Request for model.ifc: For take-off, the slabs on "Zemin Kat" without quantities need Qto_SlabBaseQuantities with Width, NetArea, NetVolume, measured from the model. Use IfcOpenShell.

First a look at what the model holds.

```python
import ifcopenshell
import ifcopenshell.util.element
import ifcopenshell.util.unit

model = ifcopenshell.open("model.ifc")
print(model.schema)
for unit_type in ("LENGTHUNIT", "AREAUNIT", "VOLUMEUNIT"):
    print(unit_type, ifcopenshell.util.unit.calculate_unit_scale(model, unit_type))
storey = next(s for s in model.by_type("IfcBuildingStorey") if s.Name == "Zemin Kat")
slabs = [e for e in ifcopenshell.util.element.get_decomposition(storey) if e.is_a("IfcSlab")]
for e in sorted(slabs, key=lambda e: e.id()):
    print(e.id(), e.is_a(), e.Name, list(ifcopenshell.util.element.get_psets(e, qtos_only=True)), sep=" | ")
```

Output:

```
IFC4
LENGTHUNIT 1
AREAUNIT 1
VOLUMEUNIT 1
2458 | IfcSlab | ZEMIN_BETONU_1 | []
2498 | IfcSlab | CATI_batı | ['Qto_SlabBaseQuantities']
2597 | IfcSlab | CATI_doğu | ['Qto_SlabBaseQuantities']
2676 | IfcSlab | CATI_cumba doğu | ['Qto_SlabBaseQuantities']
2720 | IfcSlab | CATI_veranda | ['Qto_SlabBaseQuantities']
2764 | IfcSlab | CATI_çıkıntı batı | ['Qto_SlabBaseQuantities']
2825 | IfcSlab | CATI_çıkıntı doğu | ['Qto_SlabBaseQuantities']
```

```python
import ifcopenshell
import ifcopenshell.api.pset
import ifcopenshell.geom
import ifcopenshell.util.element
import ifcopenshell.util.shape
import ifcopenshell.util.unit

model = ifcopenshell.open("model.ifc")
unit_scale = ifcopenshell.util.unit.calculate_unit_scale(model)
area_scale = ifcopenshell.util.unit.calculate_unit_scale(model, "AREAUNIT")
volume_scale = ifcopenshell.util.unit.calculate_unit_scale(model, "VOLUMEUNIT")
settings = ifcopenshell.geom.settings()

storey = next(s for s in model.by_type("IfcBuildingStorey") if s.Name == "Zemin Kat")
slabs = [e for e in ifcopenshell.util.element.get_decomposition(storey) if e.is_a("IfcSlab")]

for e in sorted(slabs, key=lambda e: e.id()):
    if ifcopenshell.util.element.get_psets(e, qtos_only=True, should_inherit=False):
        continue
    # Geometry comes back in metres, in the element's own axes.
    shape = ifcopenshell.geom.create_shape(settings, e)
    values = {
        "Width": ifcopenshell.util.shape.get_z(shape.geometry) / unit_scale,
        "NetArea": ifcopenshell.util.shape.get_footprint_area(shape.geometry) / area_scale,
        "NetVolume": ifcopenshell.util.shape.get_volume(shape.geometry) / volume_scale,
    }
    qto = ifcopenshell.api.pset.add_qto(model, product=e, name="Qto_SlabBaseQuantities")
    ifcopenshell.api.pset.edit_qto(model, qto=qto, properties=values)
    print(e.id(), {k: round(v, 3) for k, v in values.items()})

model.write("model_edited.ifc")
```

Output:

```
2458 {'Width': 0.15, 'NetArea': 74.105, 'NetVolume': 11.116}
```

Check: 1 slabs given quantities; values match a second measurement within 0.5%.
